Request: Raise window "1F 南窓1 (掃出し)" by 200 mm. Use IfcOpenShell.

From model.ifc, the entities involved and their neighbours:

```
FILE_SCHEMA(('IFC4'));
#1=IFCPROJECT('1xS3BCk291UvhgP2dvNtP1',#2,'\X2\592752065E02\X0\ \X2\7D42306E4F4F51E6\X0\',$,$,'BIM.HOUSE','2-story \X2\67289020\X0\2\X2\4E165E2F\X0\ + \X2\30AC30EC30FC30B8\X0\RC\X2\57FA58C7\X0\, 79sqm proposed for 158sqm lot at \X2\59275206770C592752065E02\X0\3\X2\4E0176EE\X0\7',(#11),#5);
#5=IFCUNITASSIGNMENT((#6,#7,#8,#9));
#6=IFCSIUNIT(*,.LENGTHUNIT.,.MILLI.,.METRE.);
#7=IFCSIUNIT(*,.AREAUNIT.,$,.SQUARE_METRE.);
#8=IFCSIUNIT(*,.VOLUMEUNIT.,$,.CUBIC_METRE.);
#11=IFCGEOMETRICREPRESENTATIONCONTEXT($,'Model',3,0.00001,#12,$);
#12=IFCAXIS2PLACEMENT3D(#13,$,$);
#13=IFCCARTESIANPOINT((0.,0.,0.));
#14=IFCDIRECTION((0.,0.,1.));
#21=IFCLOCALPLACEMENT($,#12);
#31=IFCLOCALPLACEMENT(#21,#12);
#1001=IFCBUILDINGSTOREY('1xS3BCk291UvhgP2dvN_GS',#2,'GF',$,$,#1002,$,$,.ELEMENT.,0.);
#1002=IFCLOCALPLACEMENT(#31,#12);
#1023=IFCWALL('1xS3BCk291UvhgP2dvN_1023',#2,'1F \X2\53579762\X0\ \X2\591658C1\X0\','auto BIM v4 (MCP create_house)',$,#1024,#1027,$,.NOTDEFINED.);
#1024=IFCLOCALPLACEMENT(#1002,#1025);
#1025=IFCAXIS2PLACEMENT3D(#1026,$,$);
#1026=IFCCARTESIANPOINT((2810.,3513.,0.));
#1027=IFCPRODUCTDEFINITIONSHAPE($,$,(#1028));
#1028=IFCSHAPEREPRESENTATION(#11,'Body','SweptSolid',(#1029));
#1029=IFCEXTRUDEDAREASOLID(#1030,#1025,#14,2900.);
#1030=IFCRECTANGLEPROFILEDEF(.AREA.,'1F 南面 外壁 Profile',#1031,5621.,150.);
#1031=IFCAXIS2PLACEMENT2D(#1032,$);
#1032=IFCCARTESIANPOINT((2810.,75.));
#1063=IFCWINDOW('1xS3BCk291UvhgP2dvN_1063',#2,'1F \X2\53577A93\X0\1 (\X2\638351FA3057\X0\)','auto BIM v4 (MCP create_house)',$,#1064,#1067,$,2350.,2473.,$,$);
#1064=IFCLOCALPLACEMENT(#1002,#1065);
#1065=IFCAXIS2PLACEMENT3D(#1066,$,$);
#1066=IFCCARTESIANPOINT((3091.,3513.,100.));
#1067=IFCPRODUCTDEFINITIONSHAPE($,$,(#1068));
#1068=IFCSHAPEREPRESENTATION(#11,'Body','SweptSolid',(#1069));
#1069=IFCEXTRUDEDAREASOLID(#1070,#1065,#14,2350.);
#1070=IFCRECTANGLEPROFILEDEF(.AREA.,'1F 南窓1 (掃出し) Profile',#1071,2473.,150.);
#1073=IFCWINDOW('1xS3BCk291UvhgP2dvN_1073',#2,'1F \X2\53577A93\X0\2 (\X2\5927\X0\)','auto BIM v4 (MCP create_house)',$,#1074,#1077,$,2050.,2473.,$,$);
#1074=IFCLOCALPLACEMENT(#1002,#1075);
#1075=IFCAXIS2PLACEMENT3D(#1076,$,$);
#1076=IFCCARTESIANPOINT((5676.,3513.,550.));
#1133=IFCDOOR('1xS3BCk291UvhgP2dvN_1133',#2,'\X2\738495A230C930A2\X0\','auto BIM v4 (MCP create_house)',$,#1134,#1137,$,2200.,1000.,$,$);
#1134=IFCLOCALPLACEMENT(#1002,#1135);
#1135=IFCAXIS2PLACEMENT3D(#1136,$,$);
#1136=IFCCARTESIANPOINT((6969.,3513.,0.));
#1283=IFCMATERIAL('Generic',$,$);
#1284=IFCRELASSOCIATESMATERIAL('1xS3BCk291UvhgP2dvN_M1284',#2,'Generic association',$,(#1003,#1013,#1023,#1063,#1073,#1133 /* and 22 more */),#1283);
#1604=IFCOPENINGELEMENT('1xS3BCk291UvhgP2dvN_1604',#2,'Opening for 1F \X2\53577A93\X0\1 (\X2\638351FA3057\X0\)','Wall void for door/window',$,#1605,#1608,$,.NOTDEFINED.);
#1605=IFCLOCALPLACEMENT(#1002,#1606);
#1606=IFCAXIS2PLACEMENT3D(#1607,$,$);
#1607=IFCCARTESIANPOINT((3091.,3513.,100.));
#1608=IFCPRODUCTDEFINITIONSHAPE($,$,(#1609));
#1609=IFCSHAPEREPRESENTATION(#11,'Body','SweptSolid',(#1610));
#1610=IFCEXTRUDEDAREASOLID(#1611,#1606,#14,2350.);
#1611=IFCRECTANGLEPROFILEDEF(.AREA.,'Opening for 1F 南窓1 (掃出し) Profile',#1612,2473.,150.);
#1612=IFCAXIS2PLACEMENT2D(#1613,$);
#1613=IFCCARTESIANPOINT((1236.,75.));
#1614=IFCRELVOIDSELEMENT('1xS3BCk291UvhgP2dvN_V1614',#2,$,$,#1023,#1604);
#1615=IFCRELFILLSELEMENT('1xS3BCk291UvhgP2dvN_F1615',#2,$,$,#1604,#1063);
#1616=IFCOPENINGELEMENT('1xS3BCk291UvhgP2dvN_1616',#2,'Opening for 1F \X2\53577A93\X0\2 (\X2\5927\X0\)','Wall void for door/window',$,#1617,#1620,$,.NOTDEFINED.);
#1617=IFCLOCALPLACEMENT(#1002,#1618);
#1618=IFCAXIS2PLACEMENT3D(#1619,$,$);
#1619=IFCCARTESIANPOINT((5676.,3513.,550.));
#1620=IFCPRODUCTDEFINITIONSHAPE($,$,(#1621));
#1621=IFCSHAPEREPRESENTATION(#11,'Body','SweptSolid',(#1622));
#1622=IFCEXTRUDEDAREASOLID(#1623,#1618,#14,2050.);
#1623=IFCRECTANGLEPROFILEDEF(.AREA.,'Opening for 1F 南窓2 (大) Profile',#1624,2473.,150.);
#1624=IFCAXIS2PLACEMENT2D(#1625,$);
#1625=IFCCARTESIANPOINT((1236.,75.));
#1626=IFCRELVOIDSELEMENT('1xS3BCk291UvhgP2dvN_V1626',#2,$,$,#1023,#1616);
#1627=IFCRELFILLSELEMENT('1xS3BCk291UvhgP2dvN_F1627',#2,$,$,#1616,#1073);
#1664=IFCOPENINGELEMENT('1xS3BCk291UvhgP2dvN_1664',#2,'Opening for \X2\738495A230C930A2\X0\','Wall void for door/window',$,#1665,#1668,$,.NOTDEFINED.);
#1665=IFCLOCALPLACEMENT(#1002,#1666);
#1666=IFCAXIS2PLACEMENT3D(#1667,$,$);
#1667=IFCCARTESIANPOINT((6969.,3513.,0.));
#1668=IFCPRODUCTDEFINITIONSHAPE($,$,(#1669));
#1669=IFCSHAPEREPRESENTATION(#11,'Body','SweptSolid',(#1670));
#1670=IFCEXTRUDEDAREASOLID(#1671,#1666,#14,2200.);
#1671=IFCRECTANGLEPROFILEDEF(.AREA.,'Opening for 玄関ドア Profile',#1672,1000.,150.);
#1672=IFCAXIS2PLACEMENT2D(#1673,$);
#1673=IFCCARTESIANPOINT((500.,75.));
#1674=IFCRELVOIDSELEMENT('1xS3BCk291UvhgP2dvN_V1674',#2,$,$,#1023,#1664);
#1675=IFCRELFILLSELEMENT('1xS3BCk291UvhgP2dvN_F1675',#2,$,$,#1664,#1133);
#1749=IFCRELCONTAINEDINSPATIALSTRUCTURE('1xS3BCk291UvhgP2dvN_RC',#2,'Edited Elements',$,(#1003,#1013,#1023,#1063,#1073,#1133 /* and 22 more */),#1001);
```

```python
import numpy as np
import ifcopenshell
import ifcopenshell.api.geometry
import ifcopenshell.util.placement
import ifcopenshell.util.unit

model = ifcopenshell.open("model.ifc")
unit_scale = ifcopenshell.util.unit.calculate_unit_scale(model)

window = model.by_id(1063)
opening = window.FillsVoids[0].RelatingOpeningElement
dz = 0.2 / unit_scale

shift = np.array([0.0, 0.0, dz])
# The window is not placed relative to its opening, so move both.
for product in (opening, window):
    matrix = ifcopenshell.util.placement.get_local_placement(product.ObjectPlacement)
    matrix[:3, 3] += shift
    ifcopenshell.api.geometry.edit_object_placement(model, product=product, matrix=matrix, is_si=False)

print(f"moved by {dz * unit_scale:+.3f} m")

model.write("model_updated.ifc")
```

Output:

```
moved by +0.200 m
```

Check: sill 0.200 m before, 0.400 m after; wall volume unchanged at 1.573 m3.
